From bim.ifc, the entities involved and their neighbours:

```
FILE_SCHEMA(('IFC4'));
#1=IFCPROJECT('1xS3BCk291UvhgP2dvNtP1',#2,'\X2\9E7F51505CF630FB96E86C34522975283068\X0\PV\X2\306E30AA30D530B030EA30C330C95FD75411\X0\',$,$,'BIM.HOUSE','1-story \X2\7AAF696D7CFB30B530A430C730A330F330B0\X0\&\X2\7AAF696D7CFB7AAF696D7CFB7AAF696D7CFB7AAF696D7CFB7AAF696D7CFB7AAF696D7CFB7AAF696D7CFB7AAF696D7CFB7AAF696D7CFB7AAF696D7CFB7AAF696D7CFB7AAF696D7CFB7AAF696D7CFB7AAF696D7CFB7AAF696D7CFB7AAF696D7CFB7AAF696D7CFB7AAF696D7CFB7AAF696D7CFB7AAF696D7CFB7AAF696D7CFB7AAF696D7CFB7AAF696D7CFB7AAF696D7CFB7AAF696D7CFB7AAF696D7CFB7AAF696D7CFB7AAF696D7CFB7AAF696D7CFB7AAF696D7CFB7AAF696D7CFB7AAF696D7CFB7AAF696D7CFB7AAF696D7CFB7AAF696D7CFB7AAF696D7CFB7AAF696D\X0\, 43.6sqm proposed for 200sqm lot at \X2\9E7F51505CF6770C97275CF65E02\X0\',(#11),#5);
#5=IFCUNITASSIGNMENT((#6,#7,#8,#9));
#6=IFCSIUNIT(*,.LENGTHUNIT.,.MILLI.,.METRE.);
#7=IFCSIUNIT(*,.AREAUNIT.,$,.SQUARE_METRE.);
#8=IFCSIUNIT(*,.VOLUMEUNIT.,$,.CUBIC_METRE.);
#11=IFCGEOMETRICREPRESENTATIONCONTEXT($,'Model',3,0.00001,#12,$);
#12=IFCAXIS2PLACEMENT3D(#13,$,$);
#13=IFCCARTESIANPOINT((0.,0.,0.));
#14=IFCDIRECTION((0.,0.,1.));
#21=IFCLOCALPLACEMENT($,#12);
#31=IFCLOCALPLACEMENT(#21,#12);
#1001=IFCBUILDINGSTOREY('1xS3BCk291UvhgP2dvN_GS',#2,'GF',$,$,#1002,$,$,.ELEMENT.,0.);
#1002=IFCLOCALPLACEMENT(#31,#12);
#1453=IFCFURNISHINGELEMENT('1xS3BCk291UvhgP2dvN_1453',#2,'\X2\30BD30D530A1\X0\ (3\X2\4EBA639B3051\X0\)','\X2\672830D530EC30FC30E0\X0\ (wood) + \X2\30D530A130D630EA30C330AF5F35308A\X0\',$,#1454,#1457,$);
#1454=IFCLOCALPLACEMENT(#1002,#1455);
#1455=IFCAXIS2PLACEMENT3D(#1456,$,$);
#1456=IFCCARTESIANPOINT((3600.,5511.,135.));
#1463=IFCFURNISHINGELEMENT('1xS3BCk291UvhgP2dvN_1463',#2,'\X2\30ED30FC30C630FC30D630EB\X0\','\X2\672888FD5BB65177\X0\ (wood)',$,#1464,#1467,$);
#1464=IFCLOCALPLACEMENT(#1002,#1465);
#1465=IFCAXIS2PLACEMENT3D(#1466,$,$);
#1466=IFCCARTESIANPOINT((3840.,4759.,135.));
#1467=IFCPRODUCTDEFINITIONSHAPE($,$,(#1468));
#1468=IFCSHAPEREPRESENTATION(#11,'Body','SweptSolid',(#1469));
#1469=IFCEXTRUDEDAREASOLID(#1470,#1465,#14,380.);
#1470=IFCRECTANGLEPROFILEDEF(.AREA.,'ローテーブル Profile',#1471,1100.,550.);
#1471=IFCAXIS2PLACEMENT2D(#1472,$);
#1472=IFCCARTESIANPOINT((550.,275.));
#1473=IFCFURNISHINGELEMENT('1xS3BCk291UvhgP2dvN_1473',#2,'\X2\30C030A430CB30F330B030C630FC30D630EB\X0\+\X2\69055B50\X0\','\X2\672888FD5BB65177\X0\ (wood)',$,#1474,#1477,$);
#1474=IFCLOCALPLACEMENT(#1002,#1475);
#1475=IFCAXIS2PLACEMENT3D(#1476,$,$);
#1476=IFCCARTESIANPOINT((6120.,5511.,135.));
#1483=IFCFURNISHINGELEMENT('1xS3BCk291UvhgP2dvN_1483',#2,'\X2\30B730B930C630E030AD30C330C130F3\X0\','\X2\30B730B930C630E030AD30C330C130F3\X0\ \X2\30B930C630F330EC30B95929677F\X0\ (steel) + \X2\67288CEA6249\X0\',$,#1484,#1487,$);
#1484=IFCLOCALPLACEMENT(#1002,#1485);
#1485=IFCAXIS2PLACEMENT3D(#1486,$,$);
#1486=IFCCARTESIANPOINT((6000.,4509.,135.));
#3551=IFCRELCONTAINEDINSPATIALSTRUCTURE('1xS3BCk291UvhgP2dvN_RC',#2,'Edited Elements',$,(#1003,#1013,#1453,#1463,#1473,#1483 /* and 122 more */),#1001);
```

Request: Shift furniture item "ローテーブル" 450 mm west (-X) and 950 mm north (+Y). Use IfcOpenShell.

```python
import ifcopenshell
import ifcopenshell.api.geometry
import ifcopenshell.util.placement

model = ifcopenshell.open("bim.ifc")

item = model.by_guid("1xS3BCk291UvhgP2dvN_1463")
matrix = ifcopenshell.util.placement.get_local_placement(item.ObjectPlacement)
matrix[0, 3] -= 450.0
matrix[1, 3] += 950.0
ifcopenshell.api.geometry.edit_object_placement(model, product=item, matrix=matrix, is_si=False)

print(ifcopenshell.util.placement.get_local_placement(item.ObjectPlacement).round(3) + 0.0)

model.write("bim_edited.ifc")
```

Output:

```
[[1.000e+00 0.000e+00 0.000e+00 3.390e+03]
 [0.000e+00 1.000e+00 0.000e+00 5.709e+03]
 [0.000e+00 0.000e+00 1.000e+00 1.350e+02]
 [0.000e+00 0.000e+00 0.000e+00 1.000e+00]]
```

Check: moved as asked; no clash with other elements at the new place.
